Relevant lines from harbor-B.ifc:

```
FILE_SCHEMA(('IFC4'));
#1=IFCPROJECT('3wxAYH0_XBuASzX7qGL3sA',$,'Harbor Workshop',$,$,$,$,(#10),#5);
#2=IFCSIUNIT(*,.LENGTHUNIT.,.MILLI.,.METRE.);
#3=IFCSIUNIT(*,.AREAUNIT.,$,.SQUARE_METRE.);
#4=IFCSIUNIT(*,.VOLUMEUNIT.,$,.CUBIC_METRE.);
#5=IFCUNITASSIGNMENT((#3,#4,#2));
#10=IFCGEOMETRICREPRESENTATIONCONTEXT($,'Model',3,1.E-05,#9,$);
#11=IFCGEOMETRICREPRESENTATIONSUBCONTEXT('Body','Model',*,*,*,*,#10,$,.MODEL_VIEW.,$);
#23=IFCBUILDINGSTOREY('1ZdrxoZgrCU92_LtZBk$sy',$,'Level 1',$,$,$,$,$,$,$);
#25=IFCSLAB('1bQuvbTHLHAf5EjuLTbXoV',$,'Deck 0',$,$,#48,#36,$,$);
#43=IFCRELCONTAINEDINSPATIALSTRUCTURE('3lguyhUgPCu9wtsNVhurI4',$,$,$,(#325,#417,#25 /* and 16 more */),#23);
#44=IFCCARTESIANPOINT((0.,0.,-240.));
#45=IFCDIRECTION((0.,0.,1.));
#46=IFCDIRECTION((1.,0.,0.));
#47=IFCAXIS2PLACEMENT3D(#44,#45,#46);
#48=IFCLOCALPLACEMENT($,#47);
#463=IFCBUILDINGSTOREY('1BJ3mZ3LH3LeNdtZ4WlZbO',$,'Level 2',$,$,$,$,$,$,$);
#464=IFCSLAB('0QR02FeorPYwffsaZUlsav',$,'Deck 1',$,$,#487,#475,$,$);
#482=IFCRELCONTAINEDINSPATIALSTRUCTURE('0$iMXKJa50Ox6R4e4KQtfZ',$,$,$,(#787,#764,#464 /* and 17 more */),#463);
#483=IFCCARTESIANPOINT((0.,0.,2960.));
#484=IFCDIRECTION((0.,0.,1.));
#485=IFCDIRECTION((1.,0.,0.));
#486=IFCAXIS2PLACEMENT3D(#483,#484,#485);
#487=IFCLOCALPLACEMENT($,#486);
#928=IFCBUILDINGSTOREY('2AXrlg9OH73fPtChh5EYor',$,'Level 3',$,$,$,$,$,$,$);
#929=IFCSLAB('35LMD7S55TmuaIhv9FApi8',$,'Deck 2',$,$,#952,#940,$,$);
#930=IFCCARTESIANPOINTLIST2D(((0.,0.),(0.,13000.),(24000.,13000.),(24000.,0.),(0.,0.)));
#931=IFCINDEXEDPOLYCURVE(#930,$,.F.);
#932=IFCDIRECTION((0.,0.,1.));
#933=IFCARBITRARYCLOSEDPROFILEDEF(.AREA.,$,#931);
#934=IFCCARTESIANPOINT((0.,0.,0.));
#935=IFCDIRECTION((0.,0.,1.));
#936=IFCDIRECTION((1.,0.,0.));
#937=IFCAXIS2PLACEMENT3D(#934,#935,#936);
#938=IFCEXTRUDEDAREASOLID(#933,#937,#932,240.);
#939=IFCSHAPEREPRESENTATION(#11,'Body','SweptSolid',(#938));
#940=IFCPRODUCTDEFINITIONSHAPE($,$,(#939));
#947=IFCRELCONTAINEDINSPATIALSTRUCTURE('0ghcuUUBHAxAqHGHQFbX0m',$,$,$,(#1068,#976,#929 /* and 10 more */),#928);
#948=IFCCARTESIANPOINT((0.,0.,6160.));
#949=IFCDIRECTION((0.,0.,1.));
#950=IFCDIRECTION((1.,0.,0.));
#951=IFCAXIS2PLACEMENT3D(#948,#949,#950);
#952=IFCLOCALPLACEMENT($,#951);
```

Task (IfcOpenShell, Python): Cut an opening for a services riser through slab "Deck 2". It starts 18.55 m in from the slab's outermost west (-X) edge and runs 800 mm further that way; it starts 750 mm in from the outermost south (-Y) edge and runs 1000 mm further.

```python
import numpy as np
import ifcopenshell
import ifcopenshell.api.feature
import ifcopenshell.api.geometry
import ifcopenshell.api.root
import ifcopenshell.geom
import ifcopenshell.util.placement
import ifcopenshell.util.representation
import ifcopenshell.util.shape
import ifcopenshell.util.unit

model = ifcopenshell.open("harbor-B.ifc")
unit_scale = ifcopenshell.util.unit.calculate_unit_scale(model)
settings = ifcopenshell.geom.settings()


def volume(element):
    """Net volume in cubic metres, openings subtracted."""
    shape = ifcopenshell.geom.create_shape(settings, element)
    return ifcopenshell.util.shape.get_volume(shape.geometry)


slab = model.by_guid("35LMD7S55TmuaIhv9FApi8")
before = volume(slab)

# Extent in the slab's own axes, in metres. The edges named are its -X and -Y sides.
slab_shape = ifcopenshell.geom.create_shape(settings, slab)
vertices = ifcopenshell.util.shape.get_vertices(slab_shape.geometry)
x_min, y_min, bottom = vertices.min(axis=0)
top = vertices[:, 2].max()

opening = ifcopenshell.api.root.create_entity(model, ifc_class="IfcOpeningElement", name="Services riser opening", predefined_type="OPENING")
context = ifcopenshell.util.representation.get_context(model, "Model", "Body", "MODEL_VIEW")
width, depth = 0.8, 1
outline = [(0.0, 0.0), (width, 0.0), (width, depth), (0.0, depth), (0.0, 0.0)]
# Overshoot both faces by 50 mm so the cut is clean.
shape = ifcopenshell.api.geometry.add_slab_representation(
    model, context=context, depth=top - bottom + 0.1, polyline=outline
)
ifcopenshell.api.geometry.assign_representation(model, product=opening, representation=shape)

matrix = ifcopenshell.util.placement.get_local_placement(slab.ObjectPlacement)
matrix[:, 3] = matrix @ np.append(np.array([x_min + 18.55, y_min + 0.75, bottom - 0.05]) / unit_scale, 1.0)
ifcopenshell.api.geometry.edit_object_placement(model, product=opening, matrix=matrix, is_si=False)
ifcopenshell.api.feature.add_feature(model, feature=opening, element=slab)

after = volume(slab)

print(f"slab volume {before:.3f} -> {after:.3f} m3")

model.write("harbor-B_updated.ifc")
```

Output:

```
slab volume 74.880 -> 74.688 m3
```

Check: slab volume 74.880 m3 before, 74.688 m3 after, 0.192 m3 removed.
